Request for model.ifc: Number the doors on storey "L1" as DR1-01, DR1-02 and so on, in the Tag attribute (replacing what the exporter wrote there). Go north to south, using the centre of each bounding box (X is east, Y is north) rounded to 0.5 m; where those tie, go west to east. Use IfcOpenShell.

First a look at what the model holds.

```python
import ifcopenshell
import ifcopenshell.util.element
import ifcopenshell.util.placement

model = ifcopenshell.open("model.ifc")
print(model.schema)
storey = next(s for s in model.by_type("IfcBuildingStorey") if s.Name == "L1")
doors = [e for e in ifcopenshell.util.element.get_decomposition(storey) if e.is_a("IfcDoor")]
for e in sorted(doors, key=lambda e: e.id()):
    origin = ifcopenshell.util.placement.get_local_placement(e.ObjectPlacement)[:3, 3]
    print(e.id(), e.Tag, e.Name, origin.round(2) + 0.0, sep=" | ")
```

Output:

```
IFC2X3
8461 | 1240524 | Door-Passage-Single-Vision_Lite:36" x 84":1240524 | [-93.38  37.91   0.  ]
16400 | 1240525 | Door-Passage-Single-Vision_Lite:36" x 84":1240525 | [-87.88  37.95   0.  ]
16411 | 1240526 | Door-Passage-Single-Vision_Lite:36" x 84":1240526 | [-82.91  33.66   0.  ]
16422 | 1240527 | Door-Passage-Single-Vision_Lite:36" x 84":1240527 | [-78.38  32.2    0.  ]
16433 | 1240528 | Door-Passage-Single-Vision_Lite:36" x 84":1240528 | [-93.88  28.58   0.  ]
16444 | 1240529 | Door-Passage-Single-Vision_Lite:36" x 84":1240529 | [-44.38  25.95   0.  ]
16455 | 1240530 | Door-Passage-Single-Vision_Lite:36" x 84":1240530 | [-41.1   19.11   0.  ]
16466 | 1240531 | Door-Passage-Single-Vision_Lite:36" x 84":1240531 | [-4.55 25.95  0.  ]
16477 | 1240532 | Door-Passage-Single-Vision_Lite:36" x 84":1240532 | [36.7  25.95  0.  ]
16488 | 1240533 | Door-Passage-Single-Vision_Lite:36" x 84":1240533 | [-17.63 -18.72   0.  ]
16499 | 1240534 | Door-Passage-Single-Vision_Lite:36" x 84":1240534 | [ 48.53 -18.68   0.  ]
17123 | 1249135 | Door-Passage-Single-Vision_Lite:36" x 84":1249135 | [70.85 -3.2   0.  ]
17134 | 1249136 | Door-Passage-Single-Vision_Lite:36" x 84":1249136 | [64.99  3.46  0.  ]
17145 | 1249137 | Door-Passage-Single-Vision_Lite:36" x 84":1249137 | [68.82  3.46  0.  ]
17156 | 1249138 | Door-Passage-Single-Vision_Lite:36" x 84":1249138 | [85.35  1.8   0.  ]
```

```python
import ifcopenshell
import ifcopenshell.geom
import ifcopenshell.util.element
import ifcopenshell.util.shape

model = ifcopenshell.open("model.ifc")
settings = ifcopenshell.geom.settings()
settings.set("use-world-coords", True)


def centre(element):
    shape = ifcopenshell.geom.create_shape(settings, element)
    return ifcopenshell.util.shape.get_bbox_centroid(shape.geometry)


storey = next(s for s in model.by_type("IfcBuildingStorey") if s.Name == "L1")
doors = [e for e in ifcopenshell.util.element.get_decomposition(storey) if e.is_a("IfcDoor")]

# Insertion points can sit at a corner or the storey origin, so sort by the geometry (in metres).
centres = {e: centre(e) for e in doors}
doors.sort(key=lambda e: (-round(centres[e][1] / 0.5), centres[e][0]))

for i, e in enumerate(doors, start=1):
    number = f"DR1-{i:02d}"
    e.Tag = number
    print(e.id(), number)

model.write("model_v2.ifc")
```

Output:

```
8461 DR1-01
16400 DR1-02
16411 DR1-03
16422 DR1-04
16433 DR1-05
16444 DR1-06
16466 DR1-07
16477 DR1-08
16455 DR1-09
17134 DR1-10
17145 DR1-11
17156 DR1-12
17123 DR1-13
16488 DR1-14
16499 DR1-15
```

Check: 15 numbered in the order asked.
